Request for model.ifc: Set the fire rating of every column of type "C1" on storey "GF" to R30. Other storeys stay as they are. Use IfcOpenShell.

First a look at what the model holds.

```python
import ifcopenshell
import ifcopenshell.util.element

model = ifcopenshell.open("model.ifc")
print(model.schema)
storey = next(s for s in model.by_type("IfcBuildingStorey") if s.Name == "GF")
columns = [e for e in ifcopenshell.util.element.get_decomposition(storey) if e.is_a("IfcColumn")]
seen = {}
for e in columns:
    element_type = ifcopenshell.util.element.get_type(e)
    key = (element_type.Name if element_type != e and element_type else None, ifcopenshell.util.element.get_pset(e, "Pset_ColumnCommon", "FireRating"))
    seen[key] = seen.get(key, 0) + 1
for (name, value), count in sorted(seen.items(), key=str):
    print(count, "x", name, "|", value)
```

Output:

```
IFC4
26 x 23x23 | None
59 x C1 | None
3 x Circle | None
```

```python
import ifcopenshell
import ifcopenshell.api.pset
import ifcopenshell.util.element

model = ifcopenshell.open("model.ifc")

storey = next(s for s in model.by_type("IfcBuildingStorey") if s.Name == "GF")
columns = [e for e in ifcopenshell.util.element.get_decomposition(storey) if e.is_a("IfcColumn")]

count = 0
for e in columns:
    element_type = ifcopenshell.util.element.get_type(e)
    if element_type in (None, e) or element_type.Name != "C1":
        continue
    # add_pset returns the element's existing set when there is one.
    pset = ifcopenshell.api.pset.add_pset(model, product=e, name="Pset_ColumnCommon")
    ifcopenshell.api.pset.edit_pset(model, pset=pset, properties={"FireRating": "R30"})
    count += 1

print(count, "columns updated")

model.write("model_updated.ifc")
```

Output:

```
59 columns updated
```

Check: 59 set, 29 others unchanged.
